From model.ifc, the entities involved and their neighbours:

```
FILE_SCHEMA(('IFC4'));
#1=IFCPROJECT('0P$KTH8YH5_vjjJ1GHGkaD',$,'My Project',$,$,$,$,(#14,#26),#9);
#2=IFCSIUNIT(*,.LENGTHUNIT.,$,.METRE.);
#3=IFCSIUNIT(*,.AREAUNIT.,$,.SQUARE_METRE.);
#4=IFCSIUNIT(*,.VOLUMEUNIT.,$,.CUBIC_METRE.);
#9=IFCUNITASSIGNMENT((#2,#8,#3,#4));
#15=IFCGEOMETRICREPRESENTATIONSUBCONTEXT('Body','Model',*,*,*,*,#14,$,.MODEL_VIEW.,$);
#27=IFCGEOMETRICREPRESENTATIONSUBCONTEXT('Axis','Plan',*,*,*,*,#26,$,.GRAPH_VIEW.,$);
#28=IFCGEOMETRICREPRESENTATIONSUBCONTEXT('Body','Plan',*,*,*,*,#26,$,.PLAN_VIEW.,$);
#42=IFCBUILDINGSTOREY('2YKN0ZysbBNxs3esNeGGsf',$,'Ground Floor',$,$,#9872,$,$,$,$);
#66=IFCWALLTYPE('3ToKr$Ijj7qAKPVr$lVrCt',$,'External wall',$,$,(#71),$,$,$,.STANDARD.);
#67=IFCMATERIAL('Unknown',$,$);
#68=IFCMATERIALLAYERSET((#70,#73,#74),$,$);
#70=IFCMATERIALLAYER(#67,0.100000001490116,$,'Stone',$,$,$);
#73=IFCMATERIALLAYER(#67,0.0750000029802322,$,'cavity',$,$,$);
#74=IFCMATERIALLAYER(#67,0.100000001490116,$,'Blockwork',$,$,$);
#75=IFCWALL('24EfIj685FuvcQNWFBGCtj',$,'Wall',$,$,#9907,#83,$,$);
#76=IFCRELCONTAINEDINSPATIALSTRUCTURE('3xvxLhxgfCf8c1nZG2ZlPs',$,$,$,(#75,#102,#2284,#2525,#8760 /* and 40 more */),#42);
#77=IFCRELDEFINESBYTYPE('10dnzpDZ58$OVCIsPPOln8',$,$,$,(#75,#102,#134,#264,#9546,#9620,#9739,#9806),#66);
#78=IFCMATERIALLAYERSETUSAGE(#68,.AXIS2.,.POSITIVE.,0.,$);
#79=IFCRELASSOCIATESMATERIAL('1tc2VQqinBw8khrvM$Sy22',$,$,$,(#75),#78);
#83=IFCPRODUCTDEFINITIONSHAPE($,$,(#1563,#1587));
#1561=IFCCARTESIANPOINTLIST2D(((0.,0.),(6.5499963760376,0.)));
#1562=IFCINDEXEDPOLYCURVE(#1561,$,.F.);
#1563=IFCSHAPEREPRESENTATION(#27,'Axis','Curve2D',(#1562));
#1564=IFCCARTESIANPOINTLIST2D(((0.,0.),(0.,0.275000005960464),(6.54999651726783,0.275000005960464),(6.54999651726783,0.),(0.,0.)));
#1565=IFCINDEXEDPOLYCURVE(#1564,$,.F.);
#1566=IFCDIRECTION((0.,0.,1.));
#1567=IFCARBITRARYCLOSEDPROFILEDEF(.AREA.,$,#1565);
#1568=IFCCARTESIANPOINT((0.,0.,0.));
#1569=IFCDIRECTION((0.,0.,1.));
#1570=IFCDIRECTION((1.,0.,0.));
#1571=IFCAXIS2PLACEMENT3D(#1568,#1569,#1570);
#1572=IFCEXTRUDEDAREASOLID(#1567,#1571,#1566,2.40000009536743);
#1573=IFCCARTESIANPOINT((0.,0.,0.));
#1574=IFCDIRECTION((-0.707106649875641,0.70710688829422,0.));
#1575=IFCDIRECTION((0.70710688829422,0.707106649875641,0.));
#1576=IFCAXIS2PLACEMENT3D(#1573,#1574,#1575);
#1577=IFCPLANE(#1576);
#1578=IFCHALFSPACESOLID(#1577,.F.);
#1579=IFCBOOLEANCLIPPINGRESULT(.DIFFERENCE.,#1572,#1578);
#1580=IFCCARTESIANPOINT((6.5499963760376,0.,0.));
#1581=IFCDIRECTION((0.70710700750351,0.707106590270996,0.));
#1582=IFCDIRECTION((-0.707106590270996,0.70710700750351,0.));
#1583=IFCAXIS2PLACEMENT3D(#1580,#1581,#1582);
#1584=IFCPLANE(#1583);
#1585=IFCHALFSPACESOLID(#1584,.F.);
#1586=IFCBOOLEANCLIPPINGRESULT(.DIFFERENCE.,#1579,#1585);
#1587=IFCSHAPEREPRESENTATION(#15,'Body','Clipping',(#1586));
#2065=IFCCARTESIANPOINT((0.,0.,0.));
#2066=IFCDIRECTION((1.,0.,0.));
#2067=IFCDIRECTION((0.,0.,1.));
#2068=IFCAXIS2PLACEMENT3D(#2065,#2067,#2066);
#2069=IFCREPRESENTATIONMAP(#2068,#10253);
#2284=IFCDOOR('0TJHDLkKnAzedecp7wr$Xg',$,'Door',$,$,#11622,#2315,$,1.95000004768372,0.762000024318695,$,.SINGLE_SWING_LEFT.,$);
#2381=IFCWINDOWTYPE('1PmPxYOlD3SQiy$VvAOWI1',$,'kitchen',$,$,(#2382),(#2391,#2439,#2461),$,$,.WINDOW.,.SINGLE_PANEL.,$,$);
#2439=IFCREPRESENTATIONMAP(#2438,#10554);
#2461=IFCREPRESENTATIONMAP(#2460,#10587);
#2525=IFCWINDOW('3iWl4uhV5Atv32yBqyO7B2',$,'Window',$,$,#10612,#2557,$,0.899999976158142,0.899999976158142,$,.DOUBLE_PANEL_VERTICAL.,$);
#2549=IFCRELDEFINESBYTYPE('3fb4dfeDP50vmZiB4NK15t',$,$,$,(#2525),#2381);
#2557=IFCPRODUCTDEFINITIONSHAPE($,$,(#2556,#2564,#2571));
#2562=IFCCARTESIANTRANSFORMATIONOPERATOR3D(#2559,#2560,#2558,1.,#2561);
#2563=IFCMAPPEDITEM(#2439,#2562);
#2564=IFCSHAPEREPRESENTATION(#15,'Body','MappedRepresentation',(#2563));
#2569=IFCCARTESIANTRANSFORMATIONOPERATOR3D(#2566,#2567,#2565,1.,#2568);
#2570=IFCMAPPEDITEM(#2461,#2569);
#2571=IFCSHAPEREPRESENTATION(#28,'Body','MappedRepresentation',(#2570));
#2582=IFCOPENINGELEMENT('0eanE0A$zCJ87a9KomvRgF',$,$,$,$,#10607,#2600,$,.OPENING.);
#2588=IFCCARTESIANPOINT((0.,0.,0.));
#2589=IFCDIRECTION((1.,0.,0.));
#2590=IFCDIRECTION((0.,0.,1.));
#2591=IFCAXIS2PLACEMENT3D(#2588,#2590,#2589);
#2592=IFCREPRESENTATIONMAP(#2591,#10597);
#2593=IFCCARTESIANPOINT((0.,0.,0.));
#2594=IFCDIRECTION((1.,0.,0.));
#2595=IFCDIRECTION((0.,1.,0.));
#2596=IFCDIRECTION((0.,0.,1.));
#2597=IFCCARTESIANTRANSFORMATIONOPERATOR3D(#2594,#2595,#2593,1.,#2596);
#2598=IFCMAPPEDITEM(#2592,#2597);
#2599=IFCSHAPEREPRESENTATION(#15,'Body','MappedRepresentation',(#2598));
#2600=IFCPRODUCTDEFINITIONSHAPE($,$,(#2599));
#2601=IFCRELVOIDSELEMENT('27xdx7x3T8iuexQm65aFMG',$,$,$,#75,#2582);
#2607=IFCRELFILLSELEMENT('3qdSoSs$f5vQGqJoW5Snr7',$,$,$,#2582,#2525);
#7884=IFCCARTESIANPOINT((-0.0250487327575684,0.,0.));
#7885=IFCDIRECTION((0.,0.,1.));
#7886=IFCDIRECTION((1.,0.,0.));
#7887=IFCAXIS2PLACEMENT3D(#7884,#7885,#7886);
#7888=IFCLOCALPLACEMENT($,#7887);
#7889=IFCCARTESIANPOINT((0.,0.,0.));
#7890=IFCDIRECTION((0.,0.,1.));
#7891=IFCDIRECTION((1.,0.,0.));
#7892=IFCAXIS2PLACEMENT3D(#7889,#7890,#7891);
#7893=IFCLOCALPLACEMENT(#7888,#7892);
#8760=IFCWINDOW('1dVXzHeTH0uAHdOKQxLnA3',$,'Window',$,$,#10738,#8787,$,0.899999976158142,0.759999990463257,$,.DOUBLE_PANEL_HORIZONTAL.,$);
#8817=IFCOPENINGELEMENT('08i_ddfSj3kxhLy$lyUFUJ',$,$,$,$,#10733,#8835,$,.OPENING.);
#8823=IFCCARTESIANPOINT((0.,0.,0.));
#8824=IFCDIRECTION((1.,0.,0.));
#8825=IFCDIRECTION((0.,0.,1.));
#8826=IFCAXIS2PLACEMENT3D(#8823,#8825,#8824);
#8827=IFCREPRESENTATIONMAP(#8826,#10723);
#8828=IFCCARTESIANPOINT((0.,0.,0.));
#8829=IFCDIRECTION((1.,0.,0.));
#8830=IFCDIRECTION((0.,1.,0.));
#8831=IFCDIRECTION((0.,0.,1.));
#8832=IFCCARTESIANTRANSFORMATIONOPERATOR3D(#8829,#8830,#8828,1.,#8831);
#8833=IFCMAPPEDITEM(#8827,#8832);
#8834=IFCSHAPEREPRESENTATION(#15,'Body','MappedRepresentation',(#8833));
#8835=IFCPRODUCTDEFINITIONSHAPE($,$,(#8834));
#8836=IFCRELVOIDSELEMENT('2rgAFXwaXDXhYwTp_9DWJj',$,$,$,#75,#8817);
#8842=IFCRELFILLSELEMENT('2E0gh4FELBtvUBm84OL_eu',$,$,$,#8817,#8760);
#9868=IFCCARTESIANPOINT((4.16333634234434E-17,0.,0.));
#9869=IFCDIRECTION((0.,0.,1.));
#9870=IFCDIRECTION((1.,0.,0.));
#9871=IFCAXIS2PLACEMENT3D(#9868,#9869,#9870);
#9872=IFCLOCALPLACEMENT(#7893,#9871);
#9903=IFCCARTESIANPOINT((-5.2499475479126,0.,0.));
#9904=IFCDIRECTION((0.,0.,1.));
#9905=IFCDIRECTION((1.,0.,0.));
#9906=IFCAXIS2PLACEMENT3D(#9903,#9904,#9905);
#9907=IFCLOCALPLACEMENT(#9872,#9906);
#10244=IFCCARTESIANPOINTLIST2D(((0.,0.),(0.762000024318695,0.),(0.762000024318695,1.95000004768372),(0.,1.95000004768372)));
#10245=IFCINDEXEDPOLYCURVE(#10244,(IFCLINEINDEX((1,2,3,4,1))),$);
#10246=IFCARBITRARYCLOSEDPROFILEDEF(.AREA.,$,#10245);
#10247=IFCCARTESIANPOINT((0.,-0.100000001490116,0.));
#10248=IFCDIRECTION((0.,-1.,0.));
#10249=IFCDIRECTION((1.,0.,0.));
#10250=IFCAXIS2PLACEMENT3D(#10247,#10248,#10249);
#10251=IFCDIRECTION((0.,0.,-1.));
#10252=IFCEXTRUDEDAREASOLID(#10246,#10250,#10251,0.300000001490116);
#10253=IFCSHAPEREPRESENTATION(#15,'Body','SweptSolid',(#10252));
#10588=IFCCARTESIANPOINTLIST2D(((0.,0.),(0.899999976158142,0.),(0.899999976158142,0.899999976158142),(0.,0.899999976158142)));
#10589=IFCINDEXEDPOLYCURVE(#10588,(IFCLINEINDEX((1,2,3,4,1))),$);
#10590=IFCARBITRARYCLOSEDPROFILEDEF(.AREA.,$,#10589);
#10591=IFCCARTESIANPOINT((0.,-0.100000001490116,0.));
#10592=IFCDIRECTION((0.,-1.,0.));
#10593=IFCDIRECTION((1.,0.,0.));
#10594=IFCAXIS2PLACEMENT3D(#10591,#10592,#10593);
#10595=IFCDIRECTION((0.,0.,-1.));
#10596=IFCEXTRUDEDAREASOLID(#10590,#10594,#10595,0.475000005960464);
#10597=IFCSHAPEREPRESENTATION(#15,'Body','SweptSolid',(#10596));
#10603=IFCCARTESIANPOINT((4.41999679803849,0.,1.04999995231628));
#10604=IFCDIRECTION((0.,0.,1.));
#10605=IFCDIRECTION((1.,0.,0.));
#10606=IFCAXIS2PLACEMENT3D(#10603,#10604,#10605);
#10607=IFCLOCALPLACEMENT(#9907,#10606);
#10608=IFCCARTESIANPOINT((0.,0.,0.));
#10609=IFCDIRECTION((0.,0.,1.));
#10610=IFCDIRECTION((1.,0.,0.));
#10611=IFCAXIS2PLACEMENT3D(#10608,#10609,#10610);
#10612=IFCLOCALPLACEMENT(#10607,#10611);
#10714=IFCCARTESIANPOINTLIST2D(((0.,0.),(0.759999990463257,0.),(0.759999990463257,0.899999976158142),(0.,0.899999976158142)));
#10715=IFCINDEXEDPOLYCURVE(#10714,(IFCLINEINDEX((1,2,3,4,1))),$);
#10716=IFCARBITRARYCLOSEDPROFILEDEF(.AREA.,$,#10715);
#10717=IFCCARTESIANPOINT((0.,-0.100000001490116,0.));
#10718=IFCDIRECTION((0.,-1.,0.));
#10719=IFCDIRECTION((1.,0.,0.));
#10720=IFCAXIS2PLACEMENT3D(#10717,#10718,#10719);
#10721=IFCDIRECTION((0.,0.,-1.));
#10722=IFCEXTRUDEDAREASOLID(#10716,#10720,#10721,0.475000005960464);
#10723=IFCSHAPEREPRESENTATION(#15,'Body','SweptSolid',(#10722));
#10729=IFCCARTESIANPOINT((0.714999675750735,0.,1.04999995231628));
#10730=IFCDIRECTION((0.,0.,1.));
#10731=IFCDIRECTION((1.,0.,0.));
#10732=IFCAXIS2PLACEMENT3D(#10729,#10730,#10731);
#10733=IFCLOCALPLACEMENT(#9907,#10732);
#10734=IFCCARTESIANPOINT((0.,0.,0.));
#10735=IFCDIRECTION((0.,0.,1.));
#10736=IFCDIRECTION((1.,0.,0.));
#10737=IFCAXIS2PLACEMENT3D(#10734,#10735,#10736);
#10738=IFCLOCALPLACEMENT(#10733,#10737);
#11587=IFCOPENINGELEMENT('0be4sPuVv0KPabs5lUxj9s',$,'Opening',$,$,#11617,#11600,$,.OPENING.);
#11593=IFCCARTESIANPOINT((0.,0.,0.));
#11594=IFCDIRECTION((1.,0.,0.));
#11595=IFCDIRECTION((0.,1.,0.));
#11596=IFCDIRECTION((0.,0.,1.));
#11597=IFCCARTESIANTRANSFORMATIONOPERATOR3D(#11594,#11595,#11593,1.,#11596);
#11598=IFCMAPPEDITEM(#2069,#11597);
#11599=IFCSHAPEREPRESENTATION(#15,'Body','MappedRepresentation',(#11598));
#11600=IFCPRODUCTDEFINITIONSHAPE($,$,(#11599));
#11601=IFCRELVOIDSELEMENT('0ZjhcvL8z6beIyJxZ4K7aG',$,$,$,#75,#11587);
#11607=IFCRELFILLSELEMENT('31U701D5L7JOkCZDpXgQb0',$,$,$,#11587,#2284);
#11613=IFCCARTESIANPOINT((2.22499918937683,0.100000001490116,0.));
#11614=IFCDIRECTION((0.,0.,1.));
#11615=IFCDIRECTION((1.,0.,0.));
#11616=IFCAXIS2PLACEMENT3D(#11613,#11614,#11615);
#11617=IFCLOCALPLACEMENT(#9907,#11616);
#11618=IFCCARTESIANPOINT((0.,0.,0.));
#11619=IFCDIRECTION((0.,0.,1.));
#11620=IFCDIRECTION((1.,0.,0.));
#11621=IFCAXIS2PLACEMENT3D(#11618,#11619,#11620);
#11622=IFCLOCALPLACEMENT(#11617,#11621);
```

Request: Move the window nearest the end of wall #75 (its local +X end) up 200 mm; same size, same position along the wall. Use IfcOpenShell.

```python
import numpy as np
import ifcopenshell
import ifcopenshell.api.geometry
import ifcopenshell.util.placement
import ifcopenshell.util.unit

model = ifcopenshell.open("model.ifc")
unit_scale = ifcopenshell.util.unit.calculate_unit_scale(model)

window = model.by_guid("3iWl4uhV5Atv32yBqyO7B2")
opening = window.FillsVoids[0].RelatingOpeningElement
dz = 0.2 / unit_scale

shift = np.array([0.0, 0.0, dz])
# The window is placed relative to its opening, so it follows when the opening moves.
matrix = ifcopenshell.util.placement.get_local_placement(opening.ObjectPlacement)
matrix[:3, 3] += shift
ifcopenshell.api.geometry.edit_object_placement(
    model, product=opening, matrix=matrix, is_si=False, should_transform_children=True
)

print(f"moved by {dz * unit_scale:+.3f} m")

model.write("model-out.ifc")
```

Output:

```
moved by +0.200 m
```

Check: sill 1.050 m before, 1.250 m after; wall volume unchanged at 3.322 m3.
